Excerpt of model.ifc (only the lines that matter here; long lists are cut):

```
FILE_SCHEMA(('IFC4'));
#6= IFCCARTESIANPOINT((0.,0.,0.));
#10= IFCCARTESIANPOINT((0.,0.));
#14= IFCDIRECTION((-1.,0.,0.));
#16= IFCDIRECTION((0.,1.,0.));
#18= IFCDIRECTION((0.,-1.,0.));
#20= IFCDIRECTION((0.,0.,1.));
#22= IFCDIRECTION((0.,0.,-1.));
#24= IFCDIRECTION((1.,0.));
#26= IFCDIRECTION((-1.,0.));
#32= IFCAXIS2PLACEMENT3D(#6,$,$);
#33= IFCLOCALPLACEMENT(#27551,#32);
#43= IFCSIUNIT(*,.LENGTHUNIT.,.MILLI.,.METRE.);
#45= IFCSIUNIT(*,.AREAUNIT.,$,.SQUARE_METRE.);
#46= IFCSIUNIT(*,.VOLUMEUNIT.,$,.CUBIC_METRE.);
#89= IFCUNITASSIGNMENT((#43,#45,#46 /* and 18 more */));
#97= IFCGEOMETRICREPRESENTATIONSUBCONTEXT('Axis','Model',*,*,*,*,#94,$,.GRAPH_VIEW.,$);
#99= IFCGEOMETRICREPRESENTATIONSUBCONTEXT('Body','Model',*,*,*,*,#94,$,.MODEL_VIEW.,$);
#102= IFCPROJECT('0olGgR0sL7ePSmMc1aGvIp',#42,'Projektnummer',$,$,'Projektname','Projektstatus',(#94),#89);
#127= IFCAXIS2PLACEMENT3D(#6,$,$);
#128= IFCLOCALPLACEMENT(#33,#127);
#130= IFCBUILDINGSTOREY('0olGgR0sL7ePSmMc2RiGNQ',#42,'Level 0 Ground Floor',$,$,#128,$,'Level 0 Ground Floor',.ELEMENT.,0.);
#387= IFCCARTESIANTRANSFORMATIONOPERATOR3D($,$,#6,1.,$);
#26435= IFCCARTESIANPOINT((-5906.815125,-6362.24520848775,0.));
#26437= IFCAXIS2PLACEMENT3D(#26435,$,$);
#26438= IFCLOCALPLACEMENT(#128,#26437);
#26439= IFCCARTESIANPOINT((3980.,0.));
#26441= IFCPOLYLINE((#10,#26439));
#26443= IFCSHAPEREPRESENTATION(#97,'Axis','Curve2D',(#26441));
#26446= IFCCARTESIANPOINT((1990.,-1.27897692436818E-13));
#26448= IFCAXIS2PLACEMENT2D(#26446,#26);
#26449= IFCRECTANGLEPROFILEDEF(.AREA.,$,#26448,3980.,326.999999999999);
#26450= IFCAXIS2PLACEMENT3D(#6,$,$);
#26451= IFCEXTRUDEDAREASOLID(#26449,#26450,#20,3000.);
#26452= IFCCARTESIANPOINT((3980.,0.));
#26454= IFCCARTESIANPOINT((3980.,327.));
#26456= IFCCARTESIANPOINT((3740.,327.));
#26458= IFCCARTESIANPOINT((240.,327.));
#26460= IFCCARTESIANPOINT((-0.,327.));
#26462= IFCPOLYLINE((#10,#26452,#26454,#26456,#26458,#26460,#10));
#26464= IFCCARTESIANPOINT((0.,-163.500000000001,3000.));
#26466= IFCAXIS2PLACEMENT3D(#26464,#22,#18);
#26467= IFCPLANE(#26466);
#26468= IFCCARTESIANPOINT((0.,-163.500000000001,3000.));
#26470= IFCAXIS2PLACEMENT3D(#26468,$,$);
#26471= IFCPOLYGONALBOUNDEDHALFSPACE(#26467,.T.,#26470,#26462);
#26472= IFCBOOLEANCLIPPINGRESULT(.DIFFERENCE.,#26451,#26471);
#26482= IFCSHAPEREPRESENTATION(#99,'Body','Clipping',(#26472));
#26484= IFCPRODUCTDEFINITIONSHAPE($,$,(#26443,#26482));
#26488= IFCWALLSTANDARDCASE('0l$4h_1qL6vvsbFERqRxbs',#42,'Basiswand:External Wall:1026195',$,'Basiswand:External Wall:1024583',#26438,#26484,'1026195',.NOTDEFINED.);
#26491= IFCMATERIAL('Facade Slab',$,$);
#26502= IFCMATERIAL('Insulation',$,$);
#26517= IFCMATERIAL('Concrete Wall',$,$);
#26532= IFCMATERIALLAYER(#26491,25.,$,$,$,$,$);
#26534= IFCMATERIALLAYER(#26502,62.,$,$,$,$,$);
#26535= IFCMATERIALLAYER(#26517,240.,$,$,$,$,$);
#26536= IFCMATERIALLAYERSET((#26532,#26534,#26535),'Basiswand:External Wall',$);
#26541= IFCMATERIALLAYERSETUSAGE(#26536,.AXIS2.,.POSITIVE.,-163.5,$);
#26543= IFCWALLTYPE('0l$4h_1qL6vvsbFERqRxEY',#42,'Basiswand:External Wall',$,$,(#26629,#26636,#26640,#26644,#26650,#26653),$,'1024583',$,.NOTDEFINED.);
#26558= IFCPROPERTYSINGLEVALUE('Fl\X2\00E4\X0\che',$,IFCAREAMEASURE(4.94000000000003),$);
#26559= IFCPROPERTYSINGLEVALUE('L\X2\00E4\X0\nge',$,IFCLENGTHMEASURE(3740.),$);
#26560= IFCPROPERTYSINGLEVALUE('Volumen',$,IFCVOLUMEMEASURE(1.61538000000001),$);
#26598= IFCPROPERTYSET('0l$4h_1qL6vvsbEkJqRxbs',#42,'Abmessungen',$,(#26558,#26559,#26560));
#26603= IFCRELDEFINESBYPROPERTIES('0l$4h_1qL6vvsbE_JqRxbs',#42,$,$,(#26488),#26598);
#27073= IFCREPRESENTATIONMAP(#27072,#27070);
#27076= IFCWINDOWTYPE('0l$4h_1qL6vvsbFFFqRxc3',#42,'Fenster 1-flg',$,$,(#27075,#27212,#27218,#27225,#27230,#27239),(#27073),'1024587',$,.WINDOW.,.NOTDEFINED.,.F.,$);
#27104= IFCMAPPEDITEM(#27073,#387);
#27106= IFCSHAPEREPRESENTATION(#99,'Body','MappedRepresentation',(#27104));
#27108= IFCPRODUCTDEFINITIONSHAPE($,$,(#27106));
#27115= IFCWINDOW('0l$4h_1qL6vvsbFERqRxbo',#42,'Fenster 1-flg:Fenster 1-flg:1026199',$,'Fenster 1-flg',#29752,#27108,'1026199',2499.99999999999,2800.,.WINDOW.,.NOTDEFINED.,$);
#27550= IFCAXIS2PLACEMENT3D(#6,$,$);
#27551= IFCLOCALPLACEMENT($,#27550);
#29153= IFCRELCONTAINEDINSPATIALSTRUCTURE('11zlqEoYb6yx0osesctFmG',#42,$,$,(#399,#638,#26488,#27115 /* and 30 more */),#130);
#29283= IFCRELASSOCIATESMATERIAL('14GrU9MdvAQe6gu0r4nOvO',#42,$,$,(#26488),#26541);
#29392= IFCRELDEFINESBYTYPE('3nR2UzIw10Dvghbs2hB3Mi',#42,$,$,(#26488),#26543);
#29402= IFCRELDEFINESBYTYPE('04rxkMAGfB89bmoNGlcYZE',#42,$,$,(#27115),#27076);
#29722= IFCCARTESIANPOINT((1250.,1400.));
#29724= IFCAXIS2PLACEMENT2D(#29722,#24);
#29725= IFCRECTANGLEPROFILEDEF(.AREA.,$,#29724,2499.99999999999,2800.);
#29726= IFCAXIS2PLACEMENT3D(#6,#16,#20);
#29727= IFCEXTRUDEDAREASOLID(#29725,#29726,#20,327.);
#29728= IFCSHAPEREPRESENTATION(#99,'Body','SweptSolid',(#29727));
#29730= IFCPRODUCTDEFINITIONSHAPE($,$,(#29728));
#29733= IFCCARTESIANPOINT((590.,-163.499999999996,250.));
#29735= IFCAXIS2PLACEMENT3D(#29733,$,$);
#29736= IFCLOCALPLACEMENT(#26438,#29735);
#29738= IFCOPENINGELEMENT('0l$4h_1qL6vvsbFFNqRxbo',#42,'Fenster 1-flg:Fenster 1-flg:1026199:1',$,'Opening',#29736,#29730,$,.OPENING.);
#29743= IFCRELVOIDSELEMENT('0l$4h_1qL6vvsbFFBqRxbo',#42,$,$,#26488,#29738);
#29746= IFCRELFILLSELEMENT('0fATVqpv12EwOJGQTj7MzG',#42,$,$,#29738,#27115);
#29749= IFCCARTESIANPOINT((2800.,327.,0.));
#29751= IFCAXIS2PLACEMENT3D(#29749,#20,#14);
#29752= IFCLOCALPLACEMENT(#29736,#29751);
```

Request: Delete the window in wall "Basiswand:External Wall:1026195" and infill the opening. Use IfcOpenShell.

```python
import ifcopenshell
import ifcopenshell.api.feature
import ifcopenshell.api.pset
import ifcopenshell.api.root
import ifcopenshell.geom
import ifcopenshell.util.element
import ifcopenshell.util.shape
import ifcopenshell.util.unit

model = ifcopenshell.open("model.ifc")
area_scale = ifcopenshell.util.unit.calculate_unit_scale(model, "AREAUNIT")
volume_scale = ifcopenshell.util.unit.calculate_unit_scale(model, "VOLUMEUNIT")
settings = ifcopenshell.geom.settings()


def volume(element):
    """Net volume in cubic metres, openings subtracted."""
    shape = ifcopenshell.geom.create_shape(settings, element)
    return ifcopenshell.util.shape.get_volume(shape.geometry)


window = model.by_guid("0l$4h_1qL6vvsbFERqRxbo")
opening = window.FillsVoids[0].RelatingOpeningElement
wall = opening.VoidsElements[0].RelatingBuildingElement
before = volume(wall)

ifcopenshell.api.root.remove_product(model, product=window)
ifcopenshell.api.feature.remove_feature(model, feature=opening)

after = volume(wall)
thickness = 0.327  # wall thickness in metres

# Update the wall's stored quantities.
pset = model.by_id(ifcopenshell.util.element.get_pset(wall, "Abmessungen", should_inherit=False)["id"])
ifcopenshell.api.pset.edit_pset(model, pset=pset, properties={
    "Fläche": model.create_entity("IfcAreaMeasure", after / thickness / area_scale),
    "Volumen": model.create_entity("IfcVolumeMeasure", after / volume_scale),
})

print(f"wall volume {before:.3f} -> {after:.3f} m3")

model.write("model_edited.ifc")
```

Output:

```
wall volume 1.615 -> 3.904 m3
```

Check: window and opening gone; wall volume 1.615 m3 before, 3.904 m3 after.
